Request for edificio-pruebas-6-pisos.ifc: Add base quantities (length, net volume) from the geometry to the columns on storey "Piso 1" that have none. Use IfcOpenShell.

First a look at what the model holds.

```python
import ifcopenshell
import ifcopenshell.util.element
import ifcopenshell.util.unit

model = ifcopenshell.open("edificio-pruebas-6-pisos.ifc")
print(model.schema)
for unit_type in ("LENGTHUNIT", "AREAUNIT", "VOLUMEUNIT"):
    print(unit_type, ifcopenshell.util.unit.calculate_unit_scale(model, unit_type))
storey = next(s for s in model.by_type("IfcBuildingStorey") if s.Name == "Piso 1")
columns = [e for e in ifcopenshell.util.element.get_decomposition(storey) if e.is_a("IfcColumn")]
for e in sorted(columns, key=lambda e: e.id()):
    print(e.id(), e.is_a(), e.Name, list(ifcopenshell.util.element.get_psets(e, qtos_only=True)), sep=" | ")
```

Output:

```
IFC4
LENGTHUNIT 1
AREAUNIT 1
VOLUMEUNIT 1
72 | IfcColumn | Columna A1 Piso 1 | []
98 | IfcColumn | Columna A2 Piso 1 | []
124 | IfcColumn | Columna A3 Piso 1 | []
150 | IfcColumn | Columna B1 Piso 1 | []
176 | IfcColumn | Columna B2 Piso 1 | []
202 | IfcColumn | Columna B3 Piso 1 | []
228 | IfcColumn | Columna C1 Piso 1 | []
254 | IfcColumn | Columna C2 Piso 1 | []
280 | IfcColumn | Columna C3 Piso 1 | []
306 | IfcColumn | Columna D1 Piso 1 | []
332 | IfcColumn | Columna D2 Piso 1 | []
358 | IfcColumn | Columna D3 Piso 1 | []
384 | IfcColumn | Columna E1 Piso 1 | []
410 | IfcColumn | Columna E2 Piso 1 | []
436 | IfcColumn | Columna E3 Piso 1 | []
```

```python
import ifcopenshell
import ifcopenshell.api.pset
import ifcopenshell.geom
import ifcopenshell.util.element
import ifcopenshell.util.shape
import ifcopenshell.util.unit

model = ifcopenshell.open("edificio-pruebas-6-pisos.ifc")
unit_scale = ifcopenshell.util.unit.calculate_unit_scale(model)
volume_scale = ifcopenshell.util.unit.calculate_unit_scale(model, "VOLUMEUNIT")
settings = ifcopenshell.geom.settings()

storey = next(s for s in model.by_type("IfcBuildingStorey") if s.Name == "Piso 1")
columns = [e for e in ifcopenshell.util.element.get_decomposition(storey) if e.is_a("IfcColumn")]

for e in sorted(columns, key=lambda e: e.id()):
    if ifcopenshell.util.element.get_psets(e, qtos_only=True, should_inherit=False):
        continue
    # Geometry comes back in metres, in the element's own axes.
    shape = ifcopenshell.geom.create_shape(settings, e)
    values = {
        "Length": ifcopenshell.util.shape.get_z(shape.geometry) / unit_scale,
        "NetVolume": ifcopenshell.util.shape.get_volume(shape.geometry) / volume_scale,
    }
    qto = ifcopenshell.api.pset.add_qto(model, product=e, name="Qto_ColumnBaseQuantities")
    ifcopenshell.api.pset.edit_qto(model, qto=qto, properties=values)
    print(e.id(), {k: round(v, 3) for k, v in values.items()})

model.write("edificio-pruebas-6-pisos_v2.ifc")
```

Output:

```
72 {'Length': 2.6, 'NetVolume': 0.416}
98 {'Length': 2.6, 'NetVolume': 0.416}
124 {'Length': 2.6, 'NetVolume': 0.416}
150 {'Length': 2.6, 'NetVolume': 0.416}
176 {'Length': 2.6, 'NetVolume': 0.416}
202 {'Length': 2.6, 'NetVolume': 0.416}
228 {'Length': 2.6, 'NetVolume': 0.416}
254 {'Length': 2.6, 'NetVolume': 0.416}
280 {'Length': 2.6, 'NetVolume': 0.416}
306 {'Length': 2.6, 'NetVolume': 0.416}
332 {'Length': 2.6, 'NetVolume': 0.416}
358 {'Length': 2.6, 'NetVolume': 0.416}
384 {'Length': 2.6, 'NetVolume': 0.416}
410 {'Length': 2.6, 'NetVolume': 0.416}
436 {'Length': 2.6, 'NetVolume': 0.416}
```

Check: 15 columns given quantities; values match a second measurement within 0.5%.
